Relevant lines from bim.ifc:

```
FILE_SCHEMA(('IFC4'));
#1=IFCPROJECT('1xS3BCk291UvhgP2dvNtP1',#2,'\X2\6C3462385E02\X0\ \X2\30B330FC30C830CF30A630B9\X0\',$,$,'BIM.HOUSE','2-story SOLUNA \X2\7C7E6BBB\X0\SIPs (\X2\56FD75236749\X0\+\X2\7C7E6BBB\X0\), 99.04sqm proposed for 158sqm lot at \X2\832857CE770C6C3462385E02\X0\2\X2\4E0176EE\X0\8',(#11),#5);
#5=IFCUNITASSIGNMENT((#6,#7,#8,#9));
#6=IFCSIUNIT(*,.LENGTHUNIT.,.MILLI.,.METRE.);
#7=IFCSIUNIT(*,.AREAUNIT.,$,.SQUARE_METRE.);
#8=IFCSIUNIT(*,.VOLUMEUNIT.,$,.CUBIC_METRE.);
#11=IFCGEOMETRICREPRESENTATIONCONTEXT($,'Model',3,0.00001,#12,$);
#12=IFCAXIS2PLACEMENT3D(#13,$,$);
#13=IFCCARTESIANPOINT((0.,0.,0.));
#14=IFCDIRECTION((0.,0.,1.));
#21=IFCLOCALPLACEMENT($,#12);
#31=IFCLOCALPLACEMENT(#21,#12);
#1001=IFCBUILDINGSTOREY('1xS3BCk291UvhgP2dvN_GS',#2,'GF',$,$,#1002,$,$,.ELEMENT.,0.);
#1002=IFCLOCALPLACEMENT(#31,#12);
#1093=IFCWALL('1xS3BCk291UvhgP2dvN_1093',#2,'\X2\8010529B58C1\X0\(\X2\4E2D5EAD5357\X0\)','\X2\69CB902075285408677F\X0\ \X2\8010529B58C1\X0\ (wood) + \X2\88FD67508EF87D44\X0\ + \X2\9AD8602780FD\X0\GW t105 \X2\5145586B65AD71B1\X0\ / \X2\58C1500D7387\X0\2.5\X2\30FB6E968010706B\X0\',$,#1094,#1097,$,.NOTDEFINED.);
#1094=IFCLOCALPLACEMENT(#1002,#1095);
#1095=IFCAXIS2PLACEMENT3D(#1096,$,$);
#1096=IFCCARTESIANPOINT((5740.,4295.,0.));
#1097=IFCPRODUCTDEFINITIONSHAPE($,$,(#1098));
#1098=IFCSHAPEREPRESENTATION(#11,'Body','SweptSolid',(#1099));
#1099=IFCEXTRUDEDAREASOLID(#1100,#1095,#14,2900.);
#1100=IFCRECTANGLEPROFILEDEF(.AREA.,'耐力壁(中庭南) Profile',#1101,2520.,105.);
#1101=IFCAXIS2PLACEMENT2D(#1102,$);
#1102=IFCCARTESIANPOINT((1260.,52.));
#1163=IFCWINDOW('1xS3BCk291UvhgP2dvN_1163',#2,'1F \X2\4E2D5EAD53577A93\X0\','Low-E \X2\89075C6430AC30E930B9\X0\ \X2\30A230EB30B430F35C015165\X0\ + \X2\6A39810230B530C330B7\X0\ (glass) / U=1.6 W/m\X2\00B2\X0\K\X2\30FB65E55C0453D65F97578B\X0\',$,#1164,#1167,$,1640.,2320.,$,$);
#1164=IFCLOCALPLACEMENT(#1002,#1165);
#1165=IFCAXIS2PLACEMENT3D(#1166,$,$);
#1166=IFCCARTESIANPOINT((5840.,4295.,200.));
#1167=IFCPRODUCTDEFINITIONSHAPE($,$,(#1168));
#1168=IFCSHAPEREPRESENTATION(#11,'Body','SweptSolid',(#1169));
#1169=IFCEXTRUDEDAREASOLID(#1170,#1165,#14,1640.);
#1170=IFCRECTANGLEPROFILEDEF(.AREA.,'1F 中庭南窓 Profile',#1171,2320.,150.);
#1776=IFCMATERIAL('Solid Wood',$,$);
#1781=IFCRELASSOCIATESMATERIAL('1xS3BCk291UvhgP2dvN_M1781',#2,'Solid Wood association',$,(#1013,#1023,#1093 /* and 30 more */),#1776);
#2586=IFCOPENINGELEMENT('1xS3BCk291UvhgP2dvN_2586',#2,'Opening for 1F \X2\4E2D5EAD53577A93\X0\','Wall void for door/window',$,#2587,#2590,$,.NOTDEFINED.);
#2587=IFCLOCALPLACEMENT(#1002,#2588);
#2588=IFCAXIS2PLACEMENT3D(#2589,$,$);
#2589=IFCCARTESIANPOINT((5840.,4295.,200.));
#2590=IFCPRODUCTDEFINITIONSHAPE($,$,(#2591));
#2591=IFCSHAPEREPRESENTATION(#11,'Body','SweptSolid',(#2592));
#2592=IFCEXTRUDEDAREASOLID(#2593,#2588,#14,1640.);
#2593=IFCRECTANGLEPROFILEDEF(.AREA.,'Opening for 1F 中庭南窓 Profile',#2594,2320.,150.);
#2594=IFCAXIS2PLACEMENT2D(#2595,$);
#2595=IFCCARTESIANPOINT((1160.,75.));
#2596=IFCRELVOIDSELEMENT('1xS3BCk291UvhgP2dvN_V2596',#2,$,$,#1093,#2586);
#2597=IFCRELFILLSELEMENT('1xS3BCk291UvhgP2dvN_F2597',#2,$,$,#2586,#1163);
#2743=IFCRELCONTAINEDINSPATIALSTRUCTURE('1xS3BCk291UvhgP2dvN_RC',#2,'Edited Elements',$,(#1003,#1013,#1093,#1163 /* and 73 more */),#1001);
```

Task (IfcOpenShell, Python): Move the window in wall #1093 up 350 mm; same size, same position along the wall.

```python
import numpy as np
import ifcopenshell
import ifcopenshell.api.geometry
import ifcopenshell.util.placement
import ifcopenshell.util.unit

model = ifcopenshell.open("bim.ifc")
unit_scale = ifcopenshell.util.unit.calculate_unit_scale(model)

window = model.by_guid("1xS3BCk291UvhgP2dvN_1163")
opening = window.FillsVoids[0].RelatingOpeningElement
dz = 0.35 / unit_scale

shift = np.array([0.0, 0.0, dz])
# The window is not placed relative to its opening, so move both.
for product in (opening, window):
    matrix = ifcopenshell.util.placement.get_local_placement(product.ObjectPlacement)
    matrix[:3, 3] += shift
    ifcopenshell.api.geometry.edit_object_placement(model, product=product, matrix=matrix, is_si=False)

print(f"moved by {dz * unit_scale:+.3f} m")

model.write("bim_rev.ifc")
```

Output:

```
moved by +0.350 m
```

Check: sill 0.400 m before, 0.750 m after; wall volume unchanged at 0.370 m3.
